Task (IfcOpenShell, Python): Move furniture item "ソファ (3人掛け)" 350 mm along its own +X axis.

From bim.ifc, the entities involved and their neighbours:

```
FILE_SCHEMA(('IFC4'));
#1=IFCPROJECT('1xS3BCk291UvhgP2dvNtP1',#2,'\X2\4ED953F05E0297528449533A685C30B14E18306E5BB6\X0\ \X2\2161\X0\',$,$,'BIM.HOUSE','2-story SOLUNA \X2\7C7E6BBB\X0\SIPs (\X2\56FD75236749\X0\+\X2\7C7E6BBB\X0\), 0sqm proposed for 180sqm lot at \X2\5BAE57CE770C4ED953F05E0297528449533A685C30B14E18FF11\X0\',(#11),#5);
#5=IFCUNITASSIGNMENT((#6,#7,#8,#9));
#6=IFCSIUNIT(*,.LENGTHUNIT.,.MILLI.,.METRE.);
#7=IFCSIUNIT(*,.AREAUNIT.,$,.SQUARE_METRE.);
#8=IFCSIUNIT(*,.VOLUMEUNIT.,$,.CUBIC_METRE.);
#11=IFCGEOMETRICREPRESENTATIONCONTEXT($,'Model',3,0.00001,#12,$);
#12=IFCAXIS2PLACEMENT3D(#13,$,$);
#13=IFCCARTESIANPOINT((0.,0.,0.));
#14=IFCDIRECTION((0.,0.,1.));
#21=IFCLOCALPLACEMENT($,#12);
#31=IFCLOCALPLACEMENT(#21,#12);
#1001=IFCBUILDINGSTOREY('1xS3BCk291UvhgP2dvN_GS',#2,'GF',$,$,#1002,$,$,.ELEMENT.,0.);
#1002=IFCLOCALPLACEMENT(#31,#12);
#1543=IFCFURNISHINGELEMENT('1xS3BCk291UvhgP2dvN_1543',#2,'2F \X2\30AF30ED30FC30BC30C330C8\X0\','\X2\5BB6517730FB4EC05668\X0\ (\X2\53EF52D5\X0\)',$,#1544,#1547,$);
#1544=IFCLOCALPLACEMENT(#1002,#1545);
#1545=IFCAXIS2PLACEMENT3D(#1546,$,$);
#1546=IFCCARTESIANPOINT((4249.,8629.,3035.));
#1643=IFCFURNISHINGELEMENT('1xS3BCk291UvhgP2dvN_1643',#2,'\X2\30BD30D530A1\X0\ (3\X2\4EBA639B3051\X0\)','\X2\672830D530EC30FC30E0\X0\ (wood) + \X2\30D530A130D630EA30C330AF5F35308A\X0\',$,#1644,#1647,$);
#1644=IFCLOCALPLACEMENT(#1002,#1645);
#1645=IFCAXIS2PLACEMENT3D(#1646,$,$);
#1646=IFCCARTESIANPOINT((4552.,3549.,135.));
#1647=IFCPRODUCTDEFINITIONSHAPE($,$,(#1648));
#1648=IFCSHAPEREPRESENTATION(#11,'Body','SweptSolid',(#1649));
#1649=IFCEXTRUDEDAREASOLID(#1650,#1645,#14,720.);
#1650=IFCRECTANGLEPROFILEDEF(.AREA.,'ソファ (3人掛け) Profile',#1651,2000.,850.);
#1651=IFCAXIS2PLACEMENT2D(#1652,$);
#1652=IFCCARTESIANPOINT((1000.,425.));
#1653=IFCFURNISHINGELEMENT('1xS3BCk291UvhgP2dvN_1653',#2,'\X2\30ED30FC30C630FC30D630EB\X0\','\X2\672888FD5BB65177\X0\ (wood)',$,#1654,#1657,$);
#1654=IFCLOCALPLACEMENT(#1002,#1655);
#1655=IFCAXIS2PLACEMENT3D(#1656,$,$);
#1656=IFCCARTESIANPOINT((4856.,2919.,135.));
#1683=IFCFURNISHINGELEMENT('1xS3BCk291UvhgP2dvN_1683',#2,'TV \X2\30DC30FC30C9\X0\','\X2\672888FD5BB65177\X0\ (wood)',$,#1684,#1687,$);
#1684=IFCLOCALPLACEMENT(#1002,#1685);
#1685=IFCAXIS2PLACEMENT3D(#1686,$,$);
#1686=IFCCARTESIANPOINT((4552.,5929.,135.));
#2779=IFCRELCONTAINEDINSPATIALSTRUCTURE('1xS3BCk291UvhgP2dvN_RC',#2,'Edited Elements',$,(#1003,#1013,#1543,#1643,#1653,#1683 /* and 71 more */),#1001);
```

```python
import ifcopenshell
import ifcopenshell.api.geometry
import ifcopenshell.util.placement
import ifcopenshell.util.unit

model = ifcopenshell.open("bim.ifc")
unit_scale = ifcopenshell.util.unit.calculate_unit_scale(model)

item = model.by_id(1643)
matrix = ifcopenshell.util.placement.get_local_placement(item.ObjectPlacement)
matrix[:3, 3] += matrix[:3, 0] * 0.35 / unit_scale
ifcopenshell.api.geometry.edit_object_placement(model, product=item, matrix=matrix, is_si=False)

print(ifcopenshell.util.placement.get_local_placement(item.ObjectPlacement).round(3) + 0.0)

model.write("bim_rev.ifc")
```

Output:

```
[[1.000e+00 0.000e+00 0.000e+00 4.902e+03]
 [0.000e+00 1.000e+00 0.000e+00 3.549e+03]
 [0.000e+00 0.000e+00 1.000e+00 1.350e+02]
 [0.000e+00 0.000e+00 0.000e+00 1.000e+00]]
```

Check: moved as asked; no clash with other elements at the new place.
